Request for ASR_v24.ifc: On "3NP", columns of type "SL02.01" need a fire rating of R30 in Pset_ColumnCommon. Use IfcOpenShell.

First a look at what the model holds.

```python
import ifcopenshell
import ifcopenshell.util.element

model = ifcopenshell.open("ASR_v24.ifc")
print(model.schema)
storey = next(s for s in model.by_type("IfcBuildingStorey") if s.Name == "3NP")
columns = [e for e in ifcopenshell.util.element.get_decomposition(storey) if e.is_a("IfcColumn")]
seen = {}
for e in columns:
    element_type = ifcopenshell.util.element.get_type(e)
    key = (element_type.Name if element_type != e and element_type else None, ifcopenshell.util.element.get_pset(e, "Pset_ColumnCommon", "FireRating"))
    seen[key] = seen.get(key, 0) + 1
for (name, value), count in sorted(seen.items(), key=str):
    print(count, "x", name, "|", value)
```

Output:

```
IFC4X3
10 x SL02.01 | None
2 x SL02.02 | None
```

```python
import ifcopenshell
import ifcopenshell.api.pset
import ifcopenshell.util.element

model = ifcopenshell.open("ASR_v24.ifc")

storey = next(s for s in model.by_type("IfcBuildingStorey") if s.Name == "3NP")
columns = [e for e in ifcopenshell.util.element.get_decomposition(storey) if e.is_a("IfcColumn")]

count = 0
for e in columns:
    element_type = ifcopenshell.util.element.get_type(e)
    if element_type in (None, e) or element_type.Name != "SL02.01":
        continue
    # add_pset returns the element's existing set when there is one.
    pset = ifcopenshell.api.pset.add_pset(model, product=e, name="Pset_ColumnCommon")
    ifcopenshell.api.pset.edit_pset(model, pset=pset, properties={"FireRating": "R30"})
    count += 1

print(count, "columns updated")

model.write("ASR_v24_edited.ifc")
```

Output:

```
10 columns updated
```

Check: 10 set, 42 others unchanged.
